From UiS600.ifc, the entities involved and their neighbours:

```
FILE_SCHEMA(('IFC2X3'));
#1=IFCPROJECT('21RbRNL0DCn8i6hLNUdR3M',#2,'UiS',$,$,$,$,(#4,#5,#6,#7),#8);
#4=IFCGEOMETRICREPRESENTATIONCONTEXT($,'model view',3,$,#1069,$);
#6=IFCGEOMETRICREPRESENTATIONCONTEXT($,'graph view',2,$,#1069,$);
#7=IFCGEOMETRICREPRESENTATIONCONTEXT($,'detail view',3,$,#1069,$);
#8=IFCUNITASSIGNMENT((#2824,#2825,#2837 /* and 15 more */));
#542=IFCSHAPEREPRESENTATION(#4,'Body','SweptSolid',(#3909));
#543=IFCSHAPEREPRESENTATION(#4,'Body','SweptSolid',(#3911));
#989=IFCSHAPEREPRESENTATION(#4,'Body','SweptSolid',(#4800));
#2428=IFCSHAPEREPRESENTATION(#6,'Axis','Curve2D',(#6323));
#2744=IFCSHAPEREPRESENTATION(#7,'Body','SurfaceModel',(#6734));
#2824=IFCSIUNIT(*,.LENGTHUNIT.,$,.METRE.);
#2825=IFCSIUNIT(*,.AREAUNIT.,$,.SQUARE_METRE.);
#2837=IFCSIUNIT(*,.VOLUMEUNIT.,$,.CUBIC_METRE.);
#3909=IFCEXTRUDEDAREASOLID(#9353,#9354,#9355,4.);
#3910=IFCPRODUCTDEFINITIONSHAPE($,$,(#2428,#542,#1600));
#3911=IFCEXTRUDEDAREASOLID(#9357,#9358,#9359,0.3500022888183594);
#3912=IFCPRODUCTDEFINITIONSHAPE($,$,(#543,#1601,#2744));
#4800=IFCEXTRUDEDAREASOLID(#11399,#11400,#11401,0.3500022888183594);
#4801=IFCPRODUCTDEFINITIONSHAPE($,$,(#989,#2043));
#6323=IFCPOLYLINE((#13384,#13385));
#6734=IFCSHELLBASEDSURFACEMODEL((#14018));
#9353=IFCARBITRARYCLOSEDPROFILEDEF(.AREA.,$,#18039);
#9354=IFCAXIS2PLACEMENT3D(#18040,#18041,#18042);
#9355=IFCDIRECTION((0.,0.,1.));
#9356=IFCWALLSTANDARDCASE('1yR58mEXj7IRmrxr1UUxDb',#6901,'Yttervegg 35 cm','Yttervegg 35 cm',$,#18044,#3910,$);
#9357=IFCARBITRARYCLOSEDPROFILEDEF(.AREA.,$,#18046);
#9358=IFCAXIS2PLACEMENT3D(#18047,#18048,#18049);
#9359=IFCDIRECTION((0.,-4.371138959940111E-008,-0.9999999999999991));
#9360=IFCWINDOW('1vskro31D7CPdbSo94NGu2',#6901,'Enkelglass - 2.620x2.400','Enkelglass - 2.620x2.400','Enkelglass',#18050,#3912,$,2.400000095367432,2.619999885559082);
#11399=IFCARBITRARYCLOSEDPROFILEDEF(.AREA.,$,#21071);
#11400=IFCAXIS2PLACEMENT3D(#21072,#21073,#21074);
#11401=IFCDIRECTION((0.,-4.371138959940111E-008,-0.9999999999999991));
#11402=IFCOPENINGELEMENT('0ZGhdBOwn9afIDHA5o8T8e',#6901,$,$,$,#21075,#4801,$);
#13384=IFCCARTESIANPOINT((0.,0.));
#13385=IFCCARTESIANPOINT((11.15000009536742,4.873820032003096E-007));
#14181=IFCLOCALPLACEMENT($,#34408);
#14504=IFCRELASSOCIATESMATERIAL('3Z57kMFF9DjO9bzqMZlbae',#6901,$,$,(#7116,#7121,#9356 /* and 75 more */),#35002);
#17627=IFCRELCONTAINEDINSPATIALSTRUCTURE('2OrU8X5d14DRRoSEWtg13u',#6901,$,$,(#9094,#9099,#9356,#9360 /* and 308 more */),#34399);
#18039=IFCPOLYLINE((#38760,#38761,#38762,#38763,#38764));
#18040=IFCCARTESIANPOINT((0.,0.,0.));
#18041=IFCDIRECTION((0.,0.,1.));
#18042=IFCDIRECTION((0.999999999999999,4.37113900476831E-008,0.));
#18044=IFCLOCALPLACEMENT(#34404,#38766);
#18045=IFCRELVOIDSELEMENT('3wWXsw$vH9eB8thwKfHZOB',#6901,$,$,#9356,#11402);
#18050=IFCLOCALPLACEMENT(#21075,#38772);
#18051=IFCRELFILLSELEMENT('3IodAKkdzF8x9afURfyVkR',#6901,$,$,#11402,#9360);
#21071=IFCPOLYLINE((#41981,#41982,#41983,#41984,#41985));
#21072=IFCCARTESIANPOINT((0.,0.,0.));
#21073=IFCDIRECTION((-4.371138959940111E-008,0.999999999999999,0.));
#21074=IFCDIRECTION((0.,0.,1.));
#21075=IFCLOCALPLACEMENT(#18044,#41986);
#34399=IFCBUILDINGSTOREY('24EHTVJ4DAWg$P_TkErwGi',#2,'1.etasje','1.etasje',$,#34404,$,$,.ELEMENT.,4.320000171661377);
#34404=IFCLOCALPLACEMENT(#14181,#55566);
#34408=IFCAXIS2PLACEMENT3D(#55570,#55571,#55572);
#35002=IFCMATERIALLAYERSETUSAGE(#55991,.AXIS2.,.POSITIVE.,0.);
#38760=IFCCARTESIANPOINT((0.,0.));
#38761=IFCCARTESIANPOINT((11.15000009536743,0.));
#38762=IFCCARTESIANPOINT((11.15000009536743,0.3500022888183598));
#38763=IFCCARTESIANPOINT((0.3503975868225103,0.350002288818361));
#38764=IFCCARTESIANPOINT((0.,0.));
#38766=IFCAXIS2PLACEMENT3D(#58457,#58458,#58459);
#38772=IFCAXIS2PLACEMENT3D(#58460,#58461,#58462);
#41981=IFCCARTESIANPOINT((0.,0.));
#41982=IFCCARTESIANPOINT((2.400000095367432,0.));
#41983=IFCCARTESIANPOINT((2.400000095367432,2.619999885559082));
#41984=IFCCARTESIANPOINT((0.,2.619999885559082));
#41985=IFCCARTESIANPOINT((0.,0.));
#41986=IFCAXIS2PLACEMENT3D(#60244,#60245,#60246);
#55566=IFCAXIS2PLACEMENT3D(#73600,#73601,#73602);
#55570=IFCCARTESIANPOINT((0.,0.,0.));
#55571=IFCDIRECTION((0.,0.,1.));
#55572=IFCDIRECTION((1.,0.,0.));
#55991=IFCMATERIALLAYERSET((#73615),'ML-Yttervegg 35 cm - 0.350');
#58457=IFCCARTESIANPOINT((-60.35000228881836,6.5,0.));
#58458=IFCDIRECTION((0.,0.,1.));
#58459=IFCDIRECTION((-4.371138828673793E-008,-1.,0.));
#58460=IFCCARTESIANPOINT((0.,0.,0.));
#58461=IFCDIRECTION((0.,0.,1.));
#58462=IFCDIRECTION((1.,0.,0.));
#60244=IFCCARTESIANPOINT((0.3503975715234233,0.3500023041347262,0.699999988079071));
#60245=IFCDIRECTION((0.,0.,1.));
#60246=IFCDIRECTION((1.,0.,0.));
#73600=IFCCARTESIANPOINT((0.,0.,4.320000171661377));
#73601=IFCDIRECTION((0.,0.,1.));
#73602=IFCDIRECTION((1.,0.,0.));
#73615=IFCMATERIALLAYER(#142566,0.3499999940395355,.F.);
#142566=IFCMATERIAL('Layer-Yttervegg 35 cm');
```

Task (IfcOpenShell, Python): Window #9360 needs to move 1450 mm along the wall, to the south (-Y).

```python
import ifcopenshell
import ifcopenshell.api.geometry
import ifcopenshell.util.placement
import ifcopenshell.util.unit

model = ifcopenshell.open("UiS600.ifc")
unit_scale = ifcopenshell.util.unit.calculate_unit_scale(model)

window = model.by_guid("1vskro31D7CPdbSo94NGu2")
opening = window.FillsVoids[0].RelatingOpeningElement
wall = opening.VoidsElements[0].RelatingBuildingElement

wall_matrix = ifcopenshell.util.placement.get_local_placement(wall.ObjectPlacement)
shift = wall_matrix[:3, 0] * 1.45 / unit_scale
before = ifcopenshell.util.placement.get_local_placement(window.ObjectPlacement)[:3, 3].copy()

# The window is placed relative to its opening, so it follows when the opening moves.
matrix = ifcopenshell.util.placement.get_local_placement(opening.ObjectPlacement)
matrix[:3, 3] += shift
ifcopenshell.api.geometry.edit_object_placement(
    model, product=opening, matrix=matrix, is_si=False, should_transform_children=True
)

after = ifcopenshell.util.placement.get_local_placement(window.ObjectPlacement)[:3, 3]
print("window moved by", (after - before).round(3) + 0.0)

model.write("UiS600_updated.ifc")
```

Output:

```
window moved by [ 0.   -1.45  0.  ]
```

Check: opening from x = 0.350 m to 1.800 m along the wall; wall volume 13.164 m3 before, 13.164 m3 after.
